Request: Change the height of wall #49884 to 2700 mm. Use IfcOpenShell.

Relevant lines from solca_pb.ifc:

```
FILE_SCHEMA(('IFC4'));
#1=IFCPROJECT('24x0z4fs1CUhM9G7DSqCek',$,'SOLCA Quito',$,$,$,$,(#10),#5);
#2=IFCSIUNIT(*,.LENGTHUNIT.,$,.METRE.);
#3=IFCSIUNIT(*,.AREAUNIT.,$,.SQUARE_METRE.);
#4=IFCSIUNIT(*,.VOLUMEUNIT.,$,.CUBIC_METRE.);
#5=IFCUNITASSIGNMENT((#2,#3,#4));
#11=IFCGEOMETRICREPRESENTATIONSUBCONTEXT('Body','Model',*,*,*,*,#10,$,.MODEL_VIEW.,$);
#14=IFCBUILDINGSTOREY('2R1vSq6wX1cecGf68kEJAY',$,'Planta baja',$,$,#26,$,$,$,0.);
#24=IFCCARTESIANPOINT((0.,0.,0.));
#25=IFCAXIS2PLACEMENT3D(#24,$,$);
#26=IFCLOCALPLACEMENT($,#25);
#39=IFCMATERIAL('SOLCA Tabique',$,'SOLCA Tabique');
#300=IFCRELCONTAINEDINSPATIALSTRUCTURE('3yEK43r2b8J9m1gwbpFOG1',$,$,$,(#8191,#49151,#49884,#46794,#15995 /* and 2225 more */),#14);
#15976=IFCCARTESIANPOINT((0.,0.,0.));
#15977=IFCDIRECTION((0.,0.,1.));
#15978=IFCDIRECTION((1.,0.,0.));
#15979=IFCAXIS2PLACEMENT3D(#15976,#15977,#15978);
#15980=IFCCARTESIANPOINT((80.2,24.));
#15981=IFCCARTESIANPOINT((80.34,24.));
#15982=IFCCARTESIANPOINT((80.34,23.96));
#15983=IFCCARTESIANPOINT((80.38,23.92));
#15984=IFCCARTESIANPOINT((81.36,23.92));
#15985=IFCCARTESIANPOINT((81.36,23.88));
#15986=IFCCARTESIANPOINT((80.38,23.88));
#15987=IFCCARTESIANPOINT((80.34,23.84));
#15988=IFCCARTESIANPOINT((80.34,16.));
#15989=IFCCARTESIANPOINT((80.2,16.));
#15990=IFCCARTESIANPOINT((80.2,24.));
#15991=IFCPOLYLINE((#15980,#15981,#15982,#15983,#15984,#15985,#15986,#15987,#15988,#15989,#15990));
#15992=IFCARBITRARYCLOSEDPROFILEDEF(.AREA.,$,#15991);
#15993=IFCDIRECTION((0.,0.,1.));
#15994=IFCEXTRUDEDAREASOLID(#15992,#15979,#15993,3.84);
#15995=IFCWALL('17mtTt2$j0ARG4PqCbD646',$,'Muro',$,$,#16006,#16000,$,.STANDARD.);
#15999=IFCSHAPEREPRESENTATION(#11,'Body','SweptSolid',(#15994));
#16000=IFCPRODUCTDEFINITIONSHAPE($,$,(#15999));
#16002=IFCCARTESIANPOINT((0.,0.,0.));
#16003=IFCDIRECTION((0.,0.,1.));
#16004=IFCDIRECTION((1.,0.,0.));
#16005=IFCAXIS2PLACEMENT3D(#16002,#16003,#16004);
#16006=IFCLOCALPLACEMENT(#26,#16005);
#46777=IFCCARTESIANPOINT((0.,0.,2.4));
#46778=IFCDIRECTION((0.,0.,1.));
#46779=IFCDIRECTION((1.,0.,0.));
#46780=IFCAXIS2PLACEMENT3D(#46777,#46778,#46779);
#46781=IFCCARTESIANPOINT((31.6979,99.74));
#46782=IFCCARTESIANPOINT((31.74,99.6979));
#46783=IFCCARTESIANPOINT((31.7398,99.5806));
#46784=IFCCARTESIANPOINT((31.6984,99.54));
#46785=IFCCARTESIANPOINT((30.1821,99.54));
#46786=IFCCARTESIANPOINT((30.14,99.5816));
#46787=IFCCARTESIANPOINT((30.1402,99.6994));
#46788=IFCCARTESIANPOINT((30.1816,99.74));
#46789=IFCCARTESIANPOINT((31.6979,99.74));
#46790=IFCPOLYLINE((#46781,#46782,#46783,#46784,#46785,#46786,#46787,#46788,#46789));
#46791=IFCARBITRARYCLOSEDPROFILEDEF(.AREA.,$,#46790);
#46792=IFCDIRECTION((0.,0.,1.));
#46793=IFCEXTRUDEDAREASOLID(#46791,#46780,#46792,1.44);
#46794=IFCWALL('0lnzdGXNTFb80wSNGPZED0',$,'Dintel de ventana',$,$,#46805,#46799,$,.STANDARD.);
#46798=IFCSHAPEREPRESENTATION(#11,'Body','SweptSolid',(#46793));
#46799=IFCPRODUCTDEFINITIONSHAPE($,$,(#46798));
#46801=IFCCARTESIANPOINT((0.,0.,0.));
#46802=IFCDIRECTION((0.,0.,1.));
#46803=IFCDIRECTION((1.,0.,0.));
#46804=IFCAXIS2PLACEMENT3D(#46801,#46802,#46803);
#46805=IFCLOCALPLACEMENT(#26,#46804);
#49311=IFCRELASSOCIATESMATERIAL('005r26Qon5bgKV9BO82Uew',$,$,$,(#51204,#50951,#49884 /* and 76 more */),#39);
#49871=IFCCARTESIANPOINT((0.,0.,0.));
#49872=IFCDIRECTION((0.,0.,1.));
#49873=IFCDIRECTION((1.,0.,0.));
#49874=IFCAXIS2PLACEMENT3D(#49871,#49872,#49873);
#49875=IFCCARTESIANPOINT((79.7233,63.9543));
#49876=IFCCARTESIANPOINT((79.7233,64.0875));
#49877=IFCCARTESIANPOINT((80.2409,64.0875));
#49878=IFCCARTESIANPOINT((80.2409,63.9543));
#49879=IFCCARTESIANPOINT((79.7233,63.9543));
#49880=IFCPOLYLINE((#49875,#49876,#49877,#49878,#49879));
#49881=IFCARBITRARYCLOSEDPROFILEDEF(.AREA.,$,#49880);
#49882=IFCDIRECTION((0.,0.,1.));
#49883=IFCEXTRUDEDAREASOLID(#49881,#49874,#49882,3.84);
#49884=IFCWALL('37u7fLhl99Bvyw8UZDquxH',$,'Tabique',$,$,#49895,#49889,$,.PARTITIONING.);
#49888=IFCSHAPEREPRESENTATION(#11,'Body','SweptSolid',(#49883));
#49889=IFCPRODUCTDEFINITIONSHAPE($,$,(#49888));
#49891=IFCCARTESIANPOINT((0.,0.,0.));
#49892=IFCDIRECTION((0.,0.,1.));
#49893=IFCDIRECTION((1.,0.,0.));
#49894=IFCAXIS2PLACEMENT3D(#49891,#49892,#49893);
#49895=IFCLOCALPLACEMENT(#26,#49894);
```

```python
import ifcopenshell
import ifcopenshell.geom
import ifcopenshell.util.representation
import ifcopenshell.util.shape
import ifcopenshell.util.unit

model = ifcopenshell.open("solca_pb.ifc")
unit_scale = ifcopenshell.util.unit.calculate_unit_scale(model)
settings = ifcopenshell.geom.settings()


def volume(element):
    """Net volume in cubic metres, openings subtracted."""
    shape = ifcopenshell.geom.create_shape(settings, element)
    return ifcopenshell.util.shape.get_volume(shape.geometry)


wall = model.by_guid("37u7fLhl99Bvyw8UZDquxH")
before = volume(wall)

body = ifcopenshell.util.representation.get_representation(wall, "Model", "Body")
solid = body.Items[0]
old_height = solid.Depth
solid.Depth = 2.7 / unit_scale
after = volume(wall)

print(f"height {old_height:g} -> {solid.Depth:g}, volume {before:.3f} -> {after:.3f} m3")

model.write("solca_pb_rev.ifc")
```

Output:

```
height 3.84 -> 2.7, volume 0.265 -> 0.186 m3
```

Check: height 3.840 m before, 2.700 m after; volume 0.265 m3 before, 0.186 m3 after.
